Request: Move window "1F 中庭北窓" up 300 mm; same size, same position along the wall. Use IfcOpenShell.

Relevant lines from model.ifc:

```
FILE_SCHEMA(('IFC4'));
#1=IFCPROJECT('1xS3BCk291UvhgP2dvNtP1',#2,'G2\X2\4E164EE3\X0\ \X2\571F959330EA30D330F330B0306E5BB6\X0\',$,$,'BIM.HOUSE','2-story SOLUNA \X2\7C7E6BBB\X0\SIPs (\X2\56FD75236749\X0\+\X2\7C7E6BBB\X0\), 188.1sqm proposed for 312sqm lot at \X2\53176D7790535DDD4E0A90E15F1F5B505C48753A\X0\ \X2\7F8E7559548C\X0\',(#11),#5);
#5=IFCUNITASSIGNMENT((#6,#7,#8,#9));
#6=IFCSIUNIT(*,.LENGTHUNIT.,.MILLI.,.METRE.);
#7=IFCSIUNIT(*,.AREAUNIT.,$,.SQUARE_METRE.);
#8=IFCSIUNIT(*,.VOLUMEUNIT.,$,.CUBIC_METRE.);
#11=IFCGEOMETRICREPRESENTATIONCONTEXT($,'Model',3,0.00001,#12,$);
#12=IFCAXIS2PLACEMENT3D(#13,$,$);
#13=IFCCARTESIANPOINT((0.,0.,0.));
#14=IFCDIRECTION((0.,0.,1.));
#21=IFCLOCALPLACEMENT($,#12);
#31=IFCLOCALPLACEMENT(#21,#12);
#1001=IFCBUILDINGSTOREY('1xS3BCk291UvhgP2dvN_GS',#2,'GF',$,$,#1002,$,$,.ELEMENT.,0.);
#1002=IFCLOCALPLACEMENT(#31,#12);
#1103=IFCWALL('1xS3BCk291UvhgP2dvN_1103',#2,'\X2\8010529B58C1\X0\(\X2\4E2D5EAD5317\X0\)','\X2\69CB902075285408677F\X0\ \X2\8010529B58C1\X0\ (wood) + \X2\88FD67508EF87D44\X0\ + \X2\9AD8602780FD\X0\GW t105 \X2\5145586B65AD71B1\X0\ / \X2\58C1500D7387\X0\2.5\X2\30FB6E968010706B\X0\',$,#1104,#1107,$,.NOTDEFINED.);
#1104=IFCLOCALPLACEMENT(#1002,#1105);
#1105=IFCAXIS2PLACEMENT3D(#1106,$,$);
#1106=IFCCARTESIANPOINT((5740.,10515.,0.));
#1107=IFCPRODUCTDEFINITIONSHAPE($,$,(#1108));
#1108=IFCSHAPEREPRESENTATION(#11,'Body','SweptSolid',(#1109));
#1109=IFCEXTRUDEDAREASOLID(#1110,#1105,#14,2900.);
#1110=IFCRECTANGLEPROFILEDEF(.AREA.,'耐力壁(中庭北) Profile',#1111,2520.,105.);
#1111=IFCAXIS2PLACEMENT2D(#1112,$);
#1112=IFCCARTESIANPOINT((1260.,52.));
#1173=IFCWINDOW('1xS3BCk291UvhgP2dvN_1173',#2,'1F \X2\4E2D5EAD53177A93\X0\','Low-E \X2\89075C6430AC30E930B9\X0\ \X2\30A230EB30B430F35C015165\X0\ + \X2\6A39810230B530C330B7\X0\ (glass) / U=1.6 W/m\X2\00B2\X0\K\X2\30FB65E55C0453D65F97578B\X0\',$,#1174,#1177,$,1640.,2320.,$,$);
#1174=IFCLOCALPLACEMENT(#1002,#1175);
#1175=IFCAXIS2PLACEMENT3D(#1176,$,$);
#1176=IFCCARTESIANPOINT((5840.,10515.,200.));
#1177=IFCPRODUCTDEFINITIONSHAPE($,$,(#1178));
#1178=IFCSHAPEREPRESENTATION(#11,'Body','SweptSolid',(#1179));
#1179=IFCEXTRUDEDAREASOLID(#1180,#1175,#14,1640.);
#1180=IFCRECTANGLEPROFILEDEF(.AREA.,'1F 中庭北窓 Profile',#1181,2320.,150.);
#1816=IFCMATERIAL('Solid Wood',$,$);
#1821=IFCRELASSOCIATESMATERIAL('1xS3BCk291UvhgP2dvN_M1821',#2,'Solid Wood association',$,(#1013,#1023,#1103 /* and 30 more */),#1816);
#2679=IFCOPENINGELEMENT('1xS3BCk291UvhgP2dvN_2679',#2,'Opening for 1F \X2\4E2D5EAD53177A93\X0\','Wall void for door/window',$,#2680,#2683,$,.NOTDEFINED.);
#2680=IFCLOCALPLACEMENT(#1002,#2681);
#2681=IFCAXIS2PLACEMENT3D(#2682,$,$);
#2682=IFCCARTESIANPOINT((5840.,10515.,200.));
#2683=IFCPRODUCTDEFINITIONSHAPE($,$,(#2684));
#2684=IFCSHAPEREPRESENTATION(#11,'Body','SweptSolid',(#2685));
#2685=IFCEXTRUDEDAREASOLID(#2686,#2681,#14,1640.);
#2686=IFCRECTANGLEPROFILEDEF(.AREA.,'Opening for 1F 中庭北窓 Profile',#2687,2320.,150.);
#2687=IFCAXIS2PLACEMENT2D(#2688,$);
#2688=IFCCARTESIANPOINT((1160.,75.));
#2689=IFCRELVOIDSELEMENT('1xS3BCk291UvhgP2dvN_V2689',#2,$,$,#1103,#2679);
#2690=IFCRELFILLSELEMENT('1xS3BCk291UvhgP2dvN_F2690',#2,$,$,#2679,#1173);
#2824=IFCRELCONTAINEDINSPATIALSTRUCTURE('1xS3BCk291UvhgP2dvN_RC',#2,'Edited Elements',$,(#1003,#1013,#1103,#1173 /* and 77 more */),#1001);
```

```python
import numpy as np
import ifcopenshell
import ifcopenshell.api.geometry
import ifcopenshell.util.placement
import ifcopenshell.util.unit

model = ifcopenshell.open("model.ifc")
unit_scale = ifcopenshell.util.unit.calculate_unit_scale(model)

window = model.by_guid("1xS3BCk291UvhgP2dvN_1173")
opening = window.FillsVoids[0].RelatingOpeningElement
dz = 300.0

shift = np.array([0.0, 0.0, dz])
# The window is not placed relative to its opening, so move both.
for product in (opening, window):
    matrix = ifcopenshell.util.placement.get_local_placement(product.ObjectPlacement)
    matrix[:3, 3] += shift
    ifcopenshell.api.geometry.edit_object_placement(model, product=product, matrix=matrix, is_si=False)

print(f"moved by {dz * unit_scale:+.3f} m")

model.write("model-out.ifc")
```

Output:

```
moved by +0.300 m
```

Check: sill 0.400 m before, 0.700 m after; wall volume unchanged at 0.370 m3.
